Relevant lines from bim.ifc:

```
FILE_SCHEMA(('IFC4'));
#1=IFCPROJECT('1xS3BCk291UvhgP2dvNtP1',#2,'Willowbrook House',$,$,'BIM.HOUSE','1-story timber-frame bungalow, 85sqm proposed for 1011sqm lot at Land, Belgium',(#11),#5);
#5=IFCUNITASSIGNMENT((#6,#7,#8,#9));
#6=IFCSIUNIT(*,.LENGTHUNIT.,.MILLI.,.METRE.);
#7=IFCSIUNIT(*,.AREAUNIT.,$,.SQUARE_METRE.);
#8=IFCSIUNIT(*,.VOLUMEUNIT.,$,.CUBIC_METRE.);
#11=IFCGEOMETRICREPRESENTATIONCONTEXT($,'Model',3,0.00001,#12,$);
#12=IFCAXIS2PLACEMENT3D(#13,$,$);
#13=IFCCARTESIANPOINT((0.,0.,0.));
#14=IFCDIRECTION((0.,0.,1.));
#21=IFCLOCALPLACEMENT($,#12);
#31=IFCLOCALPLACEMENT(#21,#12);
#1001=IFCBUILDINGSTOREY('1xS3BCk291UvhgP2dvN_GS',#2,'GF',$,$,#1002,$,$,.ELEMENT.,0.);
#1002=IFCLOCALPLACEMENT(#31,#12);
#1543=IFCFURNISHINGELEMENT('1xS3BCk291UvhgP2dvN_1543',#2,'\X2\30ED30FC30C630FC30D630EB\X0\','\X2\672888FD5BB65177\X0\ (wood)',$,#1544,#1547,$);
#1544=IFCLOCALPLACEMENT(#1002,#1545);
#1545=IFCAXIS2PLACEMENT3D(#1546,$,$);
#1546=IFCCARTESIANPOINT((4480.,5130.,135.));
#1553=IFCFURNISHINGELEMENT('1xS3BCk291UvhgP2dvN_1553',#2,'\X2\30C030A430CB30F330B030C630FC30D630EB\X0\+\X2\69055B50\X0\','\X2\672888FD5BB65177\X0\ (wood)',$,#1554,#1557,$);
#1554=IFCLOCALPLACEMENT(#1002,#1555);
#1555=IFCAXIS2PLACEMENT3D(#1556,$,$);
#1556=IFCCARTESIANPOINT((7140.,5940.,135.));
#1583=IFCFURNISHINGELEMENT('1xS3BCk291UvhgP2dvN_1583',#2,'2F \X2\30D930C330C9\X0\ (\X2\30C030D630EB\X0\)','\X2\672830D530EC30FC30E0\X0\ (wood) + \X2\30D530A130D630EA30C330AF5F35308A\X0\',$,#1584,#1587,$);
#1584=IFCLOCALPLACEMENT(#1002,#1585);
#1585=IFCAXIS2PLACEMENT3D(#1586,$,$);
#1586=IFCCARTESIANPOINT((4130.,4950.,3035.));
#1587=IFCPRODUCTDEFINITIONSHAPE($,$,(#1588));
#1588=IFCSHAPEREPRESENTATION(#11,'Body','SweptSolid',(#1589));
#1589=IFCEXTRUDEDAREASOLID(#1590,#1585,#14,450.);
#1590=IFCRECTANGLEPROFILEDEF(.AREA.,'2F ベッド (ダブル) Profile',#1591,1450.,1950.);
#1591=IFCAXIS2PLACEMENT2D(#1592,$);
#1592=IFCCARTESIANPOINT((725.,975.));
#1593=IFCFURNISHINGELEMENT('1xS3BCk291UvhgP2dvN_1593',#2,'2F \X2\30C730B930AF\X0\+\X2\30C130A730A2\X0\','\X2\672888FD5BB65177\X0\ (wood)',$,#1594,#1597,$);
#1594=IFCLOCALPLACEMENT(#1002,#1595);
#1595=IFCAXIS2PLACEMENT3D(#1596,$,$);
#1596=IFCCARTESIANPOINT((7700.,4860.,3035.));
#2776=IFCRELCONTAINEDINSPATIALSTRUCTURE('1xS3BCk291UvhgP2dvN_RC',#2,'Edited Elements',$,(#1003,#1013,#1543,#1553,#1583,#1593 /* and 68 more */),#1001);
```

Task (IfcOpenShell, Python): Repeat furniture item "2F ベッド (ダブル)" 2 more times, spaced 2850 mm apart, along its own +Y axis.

```python
import ifcopenshell
import ifcopenshell.api.geometry
import ifcopenshell.api.root
import ifcopenshell.util.element
import ifcopenshell.util.placement

model = ifcopenshell.open("bim.ifc")


def reuse_history(source, copy):
    """copy_class also copies each property set's owner history, people and application; keep the originals."""
    for rel in copy.IsDefinedBy:
        if rel.is_a("IfcRelDefinesByProperties") and (history := rel.RelatingPropertyDefinition.OwnerHistory):
            rel.RelatingPropertyDefinition.OwnerHistory = source.OwnerHistory
            ifcopenshell.util.element.remove_deep2(model, history)


source = model.by_id(1583)
base = ifcopenshell.util.placement.get_local_placement(source.ObjectPlacement)
step = base[:3, 1] * 2850.0

for i in range(1, 3):
    copy = ifcopenshell.api.root.copy_class(model, product=source)
    copy.Representation = ifcopenshell.util.element.copy_deep(
        model, source.Representation, exclude=["IfcGeometricRepresentationContext", "IfcRepresentationMap"]
    )
    reuse_history(source, copy)
    matrix = base.copy()
    matrix[:3, 3] += i * step
    print("added at", matrix[:3, 3].round(3) + 0.0)
    ifcopenshell.api.geometry.edit_object_placement(model, product=copy, matrix=matrix, is_si=False)

model.write("bim_updated.ifc")
```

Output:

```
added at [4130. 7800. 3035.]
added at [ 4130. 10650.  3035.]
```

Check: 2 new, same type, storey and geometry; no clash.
